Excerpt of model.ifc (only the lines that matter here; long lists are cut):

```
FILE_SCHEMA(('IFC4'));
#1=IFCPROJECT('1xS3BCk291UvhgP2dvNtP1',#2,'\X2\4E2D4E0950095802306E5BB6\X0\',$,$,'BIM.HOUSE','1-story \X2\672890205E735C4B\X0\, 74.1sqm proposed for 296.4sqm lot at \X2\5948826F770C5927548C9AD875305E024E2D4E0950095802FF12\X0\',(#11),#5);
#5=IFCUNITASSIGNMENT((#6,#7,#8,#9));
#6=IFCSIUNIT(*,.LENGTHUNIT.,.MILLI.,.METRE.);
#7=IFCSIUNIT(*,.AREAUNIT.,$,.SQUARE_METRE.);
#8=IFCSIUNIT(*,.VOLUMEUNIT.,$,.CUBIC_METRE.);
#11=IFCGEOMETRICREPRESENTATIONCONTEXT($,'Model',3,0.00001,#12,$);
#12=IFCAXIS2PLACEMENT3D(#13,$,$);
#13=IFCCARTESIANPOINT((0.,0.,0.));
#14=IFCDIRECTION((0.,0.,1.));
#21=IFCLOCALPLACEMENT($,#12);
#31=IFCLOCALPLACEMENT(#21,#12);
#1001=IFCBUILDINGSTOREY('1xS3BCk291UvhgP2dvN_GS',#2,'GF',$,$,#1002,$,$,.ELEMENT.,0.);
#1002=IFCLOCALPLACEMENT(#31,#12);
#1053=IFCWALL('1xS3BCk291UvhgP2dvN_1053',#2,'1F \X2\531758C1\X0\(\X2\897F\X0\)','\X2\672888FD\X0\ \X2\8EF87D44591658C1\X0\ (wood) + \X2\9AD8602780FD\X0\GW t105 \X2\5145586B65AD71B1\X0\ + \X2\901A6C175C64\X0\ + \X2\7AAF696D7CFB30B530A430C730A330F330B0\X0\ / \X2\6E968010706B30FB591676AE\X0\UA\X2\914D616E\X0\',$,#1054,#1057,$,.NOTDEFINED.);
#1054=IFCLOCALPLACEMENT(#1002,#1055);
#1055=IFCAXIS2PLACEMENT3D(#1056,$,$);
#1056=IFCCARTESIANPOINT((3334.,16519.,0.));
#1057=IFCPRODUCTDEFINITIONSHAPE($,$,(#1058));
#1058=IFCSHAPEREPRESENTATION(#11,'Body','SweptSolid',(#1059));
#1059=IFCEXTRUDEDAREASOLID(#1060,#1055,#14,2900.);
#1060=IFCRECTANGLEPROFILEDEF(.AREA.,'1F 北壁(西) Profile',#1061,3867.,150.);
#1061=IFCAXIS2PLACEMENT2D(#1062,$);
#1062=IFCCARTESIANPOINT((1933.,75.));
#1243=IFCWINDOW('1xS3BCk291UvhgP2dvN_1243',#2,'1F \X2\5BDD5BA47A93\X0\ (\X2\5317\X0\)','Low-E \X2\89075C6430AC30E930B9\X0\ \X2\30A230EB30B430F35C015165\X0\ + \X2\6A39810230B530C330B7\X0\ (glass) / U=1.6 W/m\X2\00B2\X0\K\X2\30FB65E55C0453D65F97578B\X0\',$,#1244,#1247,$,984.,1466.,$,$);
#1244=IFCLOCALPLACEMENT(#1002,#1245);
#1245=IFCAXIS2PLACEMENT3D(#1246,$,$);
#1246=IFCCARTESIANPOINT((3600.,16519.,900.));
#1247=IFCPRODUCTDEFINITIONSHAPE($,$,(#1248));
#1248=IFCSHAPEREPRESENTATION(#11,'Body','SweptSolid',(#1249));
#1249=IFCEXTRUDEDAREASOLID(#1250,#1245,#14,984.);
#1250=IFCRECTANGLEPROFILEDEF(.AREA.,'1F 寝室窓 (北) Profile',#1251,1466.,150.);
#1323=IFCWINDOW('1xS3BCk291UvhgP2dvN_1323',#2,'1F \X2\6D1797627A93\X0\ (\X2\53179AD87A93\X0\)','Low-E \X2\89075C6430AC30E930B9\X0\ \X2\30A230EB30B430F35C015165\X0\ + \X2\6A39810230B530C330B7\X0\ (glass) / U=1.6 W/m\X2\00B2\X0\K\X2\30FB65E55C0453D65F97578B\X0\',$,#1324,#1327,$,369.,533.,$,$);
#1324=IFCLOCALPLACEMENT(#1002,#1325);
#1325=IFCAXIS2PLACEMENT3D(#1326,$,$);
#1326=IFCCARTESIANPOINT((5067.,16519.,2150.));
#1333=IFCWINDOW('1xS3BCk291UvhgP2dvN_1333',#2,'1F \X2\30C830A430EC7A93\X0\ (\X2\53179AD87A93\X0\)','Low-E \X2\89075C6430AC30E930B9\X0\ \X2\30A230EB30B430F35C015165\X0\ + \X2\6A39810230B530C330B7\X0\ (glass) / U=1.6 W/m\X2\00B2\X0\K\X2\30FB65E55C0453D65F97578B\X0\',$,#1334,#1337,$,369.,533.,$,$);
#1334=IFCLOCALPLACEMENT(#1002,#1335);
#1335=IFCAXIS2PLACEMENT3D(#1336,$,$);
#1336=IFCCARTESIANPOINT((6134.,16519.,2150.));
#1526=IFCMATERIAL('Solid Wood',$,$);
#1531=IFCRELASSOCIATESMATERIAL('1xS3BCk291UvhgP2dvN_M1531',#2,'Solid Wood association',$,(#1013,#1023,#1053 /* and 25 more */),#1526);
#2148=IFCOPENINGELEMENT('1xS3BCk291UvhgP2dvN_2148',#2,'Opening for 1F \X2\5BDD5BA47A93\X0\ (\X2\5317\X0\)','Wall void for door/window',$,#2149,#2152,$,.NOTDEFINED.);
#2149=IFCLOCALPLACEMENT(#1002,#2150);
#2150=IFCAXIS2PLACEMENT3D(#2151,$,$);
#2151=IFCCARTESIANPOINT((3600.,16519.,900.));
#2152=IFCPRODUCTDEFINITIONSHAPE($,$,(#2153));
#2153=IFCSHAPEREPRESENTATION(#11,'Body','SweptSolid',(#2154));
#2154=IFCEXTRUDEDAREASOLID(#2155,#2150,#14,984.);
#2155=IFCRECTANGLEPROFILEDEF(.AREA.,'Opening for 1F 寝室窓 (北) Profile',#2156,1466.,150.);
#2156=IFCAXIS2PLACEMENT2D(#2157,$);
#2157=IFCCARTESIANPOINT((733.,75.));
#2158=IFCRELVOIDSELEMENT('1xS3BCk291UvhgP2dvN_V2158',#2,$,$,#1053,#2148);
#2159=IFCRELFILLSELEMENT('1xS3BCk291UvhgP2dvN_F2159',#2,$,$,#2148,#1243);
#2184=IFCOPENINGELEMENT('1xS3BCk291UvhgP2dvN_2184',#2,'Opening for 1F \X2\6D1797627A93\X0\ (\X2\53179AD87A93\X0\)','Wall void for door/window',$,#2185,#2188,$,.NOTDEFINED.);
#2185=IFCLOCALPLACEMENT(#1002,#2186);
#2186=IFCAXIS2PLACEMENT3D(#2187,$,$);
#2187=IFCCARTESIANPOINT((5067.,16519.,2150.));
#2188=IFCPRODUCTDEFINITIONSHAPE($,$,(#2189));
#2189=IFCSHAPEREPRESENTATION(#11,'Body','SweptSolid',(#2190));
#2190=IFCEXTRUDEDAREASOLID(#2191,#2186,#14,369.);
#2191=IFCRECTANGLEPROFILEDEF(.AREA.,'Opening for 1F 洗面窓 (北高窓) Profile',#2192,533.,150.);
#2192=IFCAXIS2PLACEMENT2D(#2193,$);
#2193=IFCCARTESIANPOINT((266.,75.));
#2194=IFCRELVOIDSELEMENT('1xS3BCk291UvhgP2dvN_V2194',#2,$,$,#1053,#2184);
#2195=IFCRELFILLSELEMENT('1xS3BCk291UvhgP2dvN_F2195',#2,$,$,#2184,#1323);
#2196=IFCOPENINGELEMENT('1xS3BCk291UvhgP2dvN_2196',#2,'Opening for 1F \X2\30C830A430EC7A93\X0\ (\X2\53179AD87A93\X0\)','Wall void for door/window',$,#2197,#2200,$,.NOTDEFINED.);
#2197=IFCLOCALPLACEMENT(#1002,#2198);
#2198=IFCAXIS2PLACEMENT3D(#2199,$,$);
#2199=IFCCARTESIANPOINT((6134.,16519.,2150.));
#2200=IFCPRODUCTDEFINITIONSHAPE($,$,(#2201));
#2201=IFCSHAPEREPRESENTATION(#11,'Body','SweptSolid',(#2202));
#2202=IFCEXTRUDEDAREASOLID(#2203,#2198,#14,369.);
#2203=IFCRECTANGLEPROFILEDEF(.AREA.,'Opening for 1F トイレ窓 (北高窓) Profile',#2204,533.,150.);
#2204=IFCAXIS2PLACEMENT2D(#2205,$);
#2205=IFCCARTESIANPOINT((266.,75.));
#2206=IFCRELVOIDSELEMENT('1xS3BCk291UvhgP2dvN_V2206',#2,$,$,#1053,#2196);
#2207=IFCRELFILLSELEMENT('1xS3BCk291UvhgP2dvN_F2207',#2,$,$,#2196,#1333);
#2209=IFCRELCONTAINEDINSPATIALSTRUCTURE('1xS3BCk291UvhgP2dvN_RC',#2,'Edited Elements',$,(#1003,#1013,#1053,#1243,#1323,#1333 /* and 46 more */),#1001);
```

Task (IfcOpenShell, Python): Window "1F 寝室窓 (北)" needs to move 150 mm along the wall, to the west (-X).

```python
import ifcopenshell
import ifcopenshell.api.geometry
import ifcopenshell.util.placement

model = ifcopenshell.open("model.ifc")

window = model.by_guid("1xS3BCk291UvhgP2dvN_1243")
opening = window.FillsVoids[0].RelatingOpeningElement
wall = opening.VoidsElements[0].RelatingBuildingElement

wall_matrix = ifcopenshell.util.placement.get_local_placement(wall.ObjectPlacement)
shift = wall_matrix[:3, 0] * -150.0
before = ifcopenshell.util.placement.get_local_placement(window.ObjectPlacement)[:3, 3].copy()

# The window is not placed relative to its opening, so move both.
for product in (opening, window):
    matrix = ifcopenshell.util.placement.get_local_placement(product.ObjectPlacement)
    matrix[:3, 3] += shift
    ifcopenshell.api.geometry.edit_object_placement(model, product=product, matrix=matrix, is_si=False)

after = ifcopenshell.util.placement.get_local_placement(window.ObjectPlacement)[:3, 3]
print("window moved by", (after - before).round(3) + 0.0)

model.write("model_updated.ifc")
```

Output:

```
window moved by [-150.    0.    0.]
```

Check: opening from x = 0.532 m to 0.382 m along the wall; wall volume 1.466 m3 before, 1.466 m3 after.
